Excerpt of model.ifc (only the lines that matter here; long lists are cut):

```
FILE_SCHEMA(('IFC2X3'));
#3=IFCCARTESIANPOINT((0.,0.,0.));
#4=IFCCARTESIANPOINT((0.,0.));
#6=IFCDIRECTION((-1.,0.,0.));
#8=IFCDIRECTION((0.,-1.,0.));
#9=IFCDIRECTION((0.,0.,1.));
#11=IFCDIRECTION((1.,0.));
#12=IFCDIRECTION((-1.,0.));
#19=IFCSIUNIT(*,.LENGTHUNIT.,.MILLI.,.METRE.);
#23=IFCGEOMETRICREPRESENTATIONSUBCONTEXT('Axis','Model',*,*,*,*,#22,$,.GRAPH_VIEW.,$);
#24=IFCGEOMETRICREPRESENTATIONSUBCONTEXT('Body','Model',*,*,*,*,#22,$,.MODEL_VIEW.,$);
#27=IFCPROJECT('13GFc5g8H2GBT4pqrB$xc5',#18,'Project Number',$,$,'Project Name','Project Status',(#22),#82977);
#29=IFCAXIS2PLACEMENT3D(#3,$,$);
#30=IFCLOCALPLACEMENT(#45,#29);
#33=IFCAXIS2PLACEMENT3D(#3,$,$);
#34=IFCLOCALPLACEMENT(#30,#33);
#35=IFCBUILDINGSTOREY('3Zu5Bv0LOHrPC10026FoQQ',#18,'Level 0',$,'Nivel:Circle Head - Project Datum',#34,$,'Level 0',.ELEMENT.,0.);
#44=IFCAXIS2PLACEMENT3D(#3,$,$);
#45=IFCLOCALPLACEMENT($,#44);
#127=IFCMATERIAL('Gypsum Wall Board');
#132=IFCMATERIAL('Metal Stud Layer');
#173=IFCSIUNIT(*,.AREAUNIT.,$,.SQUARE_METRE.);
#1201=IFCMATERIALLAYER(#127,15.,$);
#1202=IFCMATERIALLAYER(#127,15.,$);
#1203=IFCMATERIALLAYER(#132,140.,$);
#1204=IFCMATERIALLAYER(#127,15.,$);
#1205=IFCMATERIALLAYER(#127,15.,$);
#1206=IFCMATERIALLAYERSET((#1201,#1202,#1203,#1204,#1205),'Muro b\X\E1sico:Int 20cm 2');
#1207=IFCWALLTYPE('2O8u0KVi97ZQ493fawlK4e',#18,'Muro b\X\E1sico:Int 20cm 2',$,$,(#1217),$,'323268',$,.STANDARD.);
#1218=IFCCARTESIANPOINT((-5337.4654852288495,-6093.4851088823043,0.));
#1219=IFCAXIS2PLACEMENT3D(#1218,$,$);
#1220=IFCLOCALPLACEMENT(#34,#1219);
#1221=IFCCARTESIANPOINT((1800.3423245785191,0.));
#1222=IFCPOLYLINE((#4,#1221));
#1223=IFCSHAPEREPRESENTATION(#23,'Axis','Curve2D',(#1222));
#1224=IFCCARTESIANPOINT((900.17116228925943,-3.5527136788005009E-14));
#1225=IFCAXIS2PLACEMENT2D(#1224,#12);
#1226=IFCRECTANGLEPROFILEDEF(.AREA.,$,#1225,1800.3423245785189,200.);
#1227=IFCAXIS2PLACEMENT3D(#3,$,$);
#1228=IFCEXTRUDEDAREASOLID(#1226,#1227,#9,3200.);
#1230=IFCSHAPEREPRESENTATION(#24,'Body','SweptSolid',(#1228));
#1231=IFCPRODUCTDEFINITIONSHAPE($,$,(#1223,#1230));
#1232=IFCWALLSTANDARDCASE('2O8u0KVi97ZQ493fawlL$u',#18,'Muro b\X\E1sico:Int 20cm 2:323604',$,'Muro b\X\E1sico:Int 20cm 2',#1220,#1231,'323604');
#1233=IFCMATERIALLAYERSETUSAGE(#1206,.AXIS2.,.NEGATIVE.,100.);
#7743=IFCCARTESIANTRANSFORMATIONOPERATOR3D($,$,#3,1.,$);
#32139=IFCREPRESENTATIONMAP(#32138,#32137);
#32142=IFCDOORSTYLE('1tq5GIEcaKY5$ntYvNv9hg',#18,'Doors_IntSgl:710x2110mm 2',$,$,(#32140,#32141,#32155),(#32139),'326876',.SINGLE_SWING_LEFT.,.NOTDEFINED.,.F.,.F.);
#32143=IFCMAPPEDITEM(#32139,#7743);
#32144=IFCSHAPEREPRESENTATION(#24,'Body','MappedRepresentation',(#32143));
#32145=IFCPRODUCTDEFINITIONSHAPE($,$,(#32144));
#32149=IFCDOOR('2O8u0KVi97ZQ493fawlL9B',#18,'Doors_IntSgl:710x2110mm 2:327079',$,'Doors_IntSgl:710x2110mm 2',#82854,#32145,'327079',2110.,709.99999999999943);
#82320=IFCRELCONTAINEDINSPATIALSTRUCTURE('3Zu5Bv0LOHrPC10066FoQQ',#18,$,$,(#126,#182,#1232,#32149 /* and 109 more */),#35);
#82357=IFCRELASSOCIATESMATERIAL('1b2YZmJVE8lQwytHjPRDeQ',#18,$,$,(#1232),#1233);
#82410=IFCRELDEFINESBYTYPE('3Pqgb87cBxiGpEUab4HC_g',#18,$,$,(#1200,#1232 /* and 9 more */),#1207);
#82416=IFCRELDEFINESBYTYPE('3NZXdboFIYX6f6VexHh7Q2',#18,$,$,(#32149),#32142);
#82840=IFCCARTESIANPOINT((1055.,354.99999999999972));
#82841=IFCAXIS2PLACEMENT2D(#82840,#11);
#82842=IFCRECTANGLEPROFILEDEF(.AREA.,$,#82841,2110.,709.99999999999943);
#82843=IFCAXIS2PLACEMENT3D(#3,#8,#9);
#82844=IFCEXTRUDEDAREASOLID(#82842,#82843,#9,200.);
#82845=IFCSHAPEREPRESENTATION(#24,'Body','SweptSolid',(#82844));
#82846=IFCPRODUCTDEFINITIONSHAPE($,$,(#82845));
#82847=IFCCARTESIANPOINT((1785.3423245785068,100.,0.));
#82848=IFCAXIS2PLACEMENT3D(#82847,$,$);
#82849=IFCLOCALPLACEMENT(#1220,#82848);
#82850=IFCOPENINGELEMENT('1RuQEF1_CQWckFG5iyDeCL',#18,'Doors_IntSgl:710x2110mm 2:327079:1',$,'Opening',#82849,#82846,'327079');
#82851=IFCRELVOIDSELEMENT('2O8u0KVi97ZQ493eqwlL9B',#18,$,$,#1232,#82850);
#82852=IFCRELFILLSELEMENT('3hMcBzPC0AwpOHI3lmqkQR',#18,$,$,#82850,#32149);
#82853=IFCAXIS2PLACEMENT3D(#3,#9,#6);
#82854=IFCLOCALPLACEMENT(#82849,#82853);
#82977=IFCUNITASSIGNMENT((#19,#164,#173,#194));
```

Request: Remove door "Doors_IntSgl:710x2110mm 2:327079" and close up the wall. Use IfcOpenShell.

```python
import ifcopenshell
import ifcopenshell.api.feature
import ifcopenshell.api.root
import ifcopenshell.geom
import ifcopenshell.util.shape

model = ifcopenshell.open("model.ifc")
settings = ifcopenshell.geom.settings()


def volume(element):
    """Net volume in cubic metres, openings subtracted."""
    shape = ifcopenshell.geom.create_shape(settings, element)
    return ifcopenshell.util.shape.get_volume(shape.geometry)


door = model.by_id(32149)
opening = door.FillsVoids[0].RelatingOpeningElement
wall = opening.VoidsElements[0].RelatingBuildingElement
before = volume(wall)

ifcopenshell.api.root.remove_product(model, product=door)
ifcopenshell.api.feature.remove_feature(model, feature=opening)

after = volume(wall)

print(f"wall volume {before:.3f} -> {after:.3f} m3")

model.write("model_updated.ifc")
```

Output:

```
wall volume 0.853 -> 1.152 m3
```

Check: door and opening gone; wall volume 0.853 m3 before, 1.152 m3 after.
